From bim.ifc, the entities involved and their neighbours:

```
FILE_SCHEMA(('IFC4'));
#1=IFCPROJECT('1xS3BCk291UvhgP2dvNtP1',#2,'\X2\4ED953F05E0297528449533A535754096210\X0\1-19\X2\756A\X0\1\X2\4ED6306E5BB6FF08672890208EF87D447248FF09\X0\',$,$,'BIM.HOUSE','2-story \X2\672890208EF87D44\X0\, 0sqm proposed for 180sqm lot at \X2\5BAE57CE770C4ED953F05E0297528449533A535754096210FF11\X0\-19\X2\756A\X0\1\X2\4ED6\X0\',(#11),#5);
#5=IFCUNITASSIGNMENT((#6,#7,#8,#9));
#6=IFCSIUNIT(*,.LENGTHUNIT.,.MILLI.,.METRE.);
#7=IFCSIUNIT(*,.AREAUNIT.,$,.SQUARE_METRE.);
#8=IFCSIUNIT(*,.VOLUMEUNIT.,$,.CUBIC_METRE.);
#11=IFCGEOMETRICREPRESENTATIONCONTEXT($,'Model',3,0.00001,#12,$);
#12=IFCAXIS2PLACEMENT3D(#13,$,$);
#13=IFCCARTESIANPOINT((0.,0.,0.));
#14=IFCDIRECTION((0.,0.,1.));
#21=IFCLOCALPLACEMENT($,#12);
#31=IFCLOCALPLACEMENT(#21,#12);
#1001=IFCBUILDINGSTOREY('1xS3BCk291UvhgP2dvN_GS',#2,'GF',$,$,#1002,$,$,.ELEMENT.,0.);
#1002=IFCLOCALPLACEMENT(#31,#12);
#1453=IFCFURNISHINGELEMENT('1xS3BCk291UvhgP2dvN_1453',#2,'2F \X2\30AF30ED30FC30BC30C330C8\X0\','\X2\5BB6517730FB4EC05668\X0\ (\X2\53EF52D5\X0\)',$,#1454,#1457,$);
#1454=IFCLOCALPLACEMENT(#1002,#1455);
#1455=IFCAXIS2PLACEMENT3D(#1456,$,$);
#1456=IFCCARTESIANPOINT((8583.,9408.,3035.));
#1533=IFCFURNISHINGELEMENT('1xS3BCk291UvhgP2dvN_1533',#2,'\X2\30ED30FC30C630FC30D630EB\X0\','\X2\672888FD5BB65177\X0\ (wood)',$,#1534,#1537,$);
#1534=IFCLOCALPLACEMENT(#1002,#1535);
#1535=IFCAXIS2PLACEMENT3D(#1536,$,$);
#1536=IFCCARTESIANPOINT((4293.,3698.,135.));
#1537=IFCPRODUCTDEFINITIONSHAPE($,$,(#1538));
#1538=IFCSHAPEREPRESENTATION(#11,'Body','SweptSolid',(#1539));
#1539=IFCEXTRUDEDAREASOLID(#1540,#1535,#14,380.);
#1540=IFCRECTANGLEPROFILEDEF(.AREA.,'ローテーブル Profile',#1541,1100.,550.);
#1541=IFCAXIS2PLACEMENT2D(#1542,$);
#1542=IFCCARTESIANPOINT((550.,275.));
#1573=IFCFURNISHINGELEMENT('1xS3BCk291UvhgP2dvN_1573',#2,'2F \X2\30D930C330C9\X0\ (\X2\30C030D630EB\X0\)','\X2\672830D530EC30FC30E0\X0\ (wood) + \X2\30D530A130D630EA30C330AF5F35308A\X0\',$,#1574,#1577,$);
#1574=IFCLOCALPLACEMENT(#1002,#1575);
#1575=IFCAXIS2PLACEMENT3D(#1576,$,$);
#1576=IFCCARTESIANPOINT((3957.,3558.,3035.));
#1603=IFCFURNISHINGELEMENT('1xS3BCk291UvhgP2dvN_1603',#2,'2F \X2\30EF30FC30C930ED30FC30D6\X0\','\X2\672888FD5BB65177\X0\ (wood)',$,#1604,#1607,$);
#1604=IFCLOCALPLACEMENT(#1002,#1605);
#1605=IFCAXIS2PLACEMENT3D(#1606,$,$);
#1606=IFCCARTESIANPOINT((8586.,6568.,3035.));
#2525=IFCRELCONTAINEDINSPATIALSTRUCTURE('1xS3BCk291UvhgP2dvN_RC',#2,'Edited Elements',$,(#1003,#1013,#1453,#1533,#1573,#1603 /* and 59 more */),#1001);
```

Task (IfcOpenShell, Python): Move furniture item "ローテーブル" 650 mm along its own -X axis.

```python
import ifcopenshell
import ifcopenshell.api.geometry
import ifcopenshell.util.placement
import ifcopenshell.util.unit

model = ifcopenshell.open("bim.ifc")
unit_scale = ifcopenshell.util.unit.calculate_unit_scale(model)

item = model.by_guid("1xS3BCk291UvhgP2dvN_1533")
matrix = ifcopenshell.util.placement.get_local_placement(item.ObjectPlacement)
matrix[:3, 3] -= matrix[:3, 0] * 0.65 / unit_scale
ifcopenshell.api.geometry.edit_object_placement(model, product=item, matrix=matrix, is_si=False)

print(ifcopenshell.util.placement.get_local_placement(item.ObjectPlacement).round(3) + 0.0)

model.write("bim_edited.ifc")
```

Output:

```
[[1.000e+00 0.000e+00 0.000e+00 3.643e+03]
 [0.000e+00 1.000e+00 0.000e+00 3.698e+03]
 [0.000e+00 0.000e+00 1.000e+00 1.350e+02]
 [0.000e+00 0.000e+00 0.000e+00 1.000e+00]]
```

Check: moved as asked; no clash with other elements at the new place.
